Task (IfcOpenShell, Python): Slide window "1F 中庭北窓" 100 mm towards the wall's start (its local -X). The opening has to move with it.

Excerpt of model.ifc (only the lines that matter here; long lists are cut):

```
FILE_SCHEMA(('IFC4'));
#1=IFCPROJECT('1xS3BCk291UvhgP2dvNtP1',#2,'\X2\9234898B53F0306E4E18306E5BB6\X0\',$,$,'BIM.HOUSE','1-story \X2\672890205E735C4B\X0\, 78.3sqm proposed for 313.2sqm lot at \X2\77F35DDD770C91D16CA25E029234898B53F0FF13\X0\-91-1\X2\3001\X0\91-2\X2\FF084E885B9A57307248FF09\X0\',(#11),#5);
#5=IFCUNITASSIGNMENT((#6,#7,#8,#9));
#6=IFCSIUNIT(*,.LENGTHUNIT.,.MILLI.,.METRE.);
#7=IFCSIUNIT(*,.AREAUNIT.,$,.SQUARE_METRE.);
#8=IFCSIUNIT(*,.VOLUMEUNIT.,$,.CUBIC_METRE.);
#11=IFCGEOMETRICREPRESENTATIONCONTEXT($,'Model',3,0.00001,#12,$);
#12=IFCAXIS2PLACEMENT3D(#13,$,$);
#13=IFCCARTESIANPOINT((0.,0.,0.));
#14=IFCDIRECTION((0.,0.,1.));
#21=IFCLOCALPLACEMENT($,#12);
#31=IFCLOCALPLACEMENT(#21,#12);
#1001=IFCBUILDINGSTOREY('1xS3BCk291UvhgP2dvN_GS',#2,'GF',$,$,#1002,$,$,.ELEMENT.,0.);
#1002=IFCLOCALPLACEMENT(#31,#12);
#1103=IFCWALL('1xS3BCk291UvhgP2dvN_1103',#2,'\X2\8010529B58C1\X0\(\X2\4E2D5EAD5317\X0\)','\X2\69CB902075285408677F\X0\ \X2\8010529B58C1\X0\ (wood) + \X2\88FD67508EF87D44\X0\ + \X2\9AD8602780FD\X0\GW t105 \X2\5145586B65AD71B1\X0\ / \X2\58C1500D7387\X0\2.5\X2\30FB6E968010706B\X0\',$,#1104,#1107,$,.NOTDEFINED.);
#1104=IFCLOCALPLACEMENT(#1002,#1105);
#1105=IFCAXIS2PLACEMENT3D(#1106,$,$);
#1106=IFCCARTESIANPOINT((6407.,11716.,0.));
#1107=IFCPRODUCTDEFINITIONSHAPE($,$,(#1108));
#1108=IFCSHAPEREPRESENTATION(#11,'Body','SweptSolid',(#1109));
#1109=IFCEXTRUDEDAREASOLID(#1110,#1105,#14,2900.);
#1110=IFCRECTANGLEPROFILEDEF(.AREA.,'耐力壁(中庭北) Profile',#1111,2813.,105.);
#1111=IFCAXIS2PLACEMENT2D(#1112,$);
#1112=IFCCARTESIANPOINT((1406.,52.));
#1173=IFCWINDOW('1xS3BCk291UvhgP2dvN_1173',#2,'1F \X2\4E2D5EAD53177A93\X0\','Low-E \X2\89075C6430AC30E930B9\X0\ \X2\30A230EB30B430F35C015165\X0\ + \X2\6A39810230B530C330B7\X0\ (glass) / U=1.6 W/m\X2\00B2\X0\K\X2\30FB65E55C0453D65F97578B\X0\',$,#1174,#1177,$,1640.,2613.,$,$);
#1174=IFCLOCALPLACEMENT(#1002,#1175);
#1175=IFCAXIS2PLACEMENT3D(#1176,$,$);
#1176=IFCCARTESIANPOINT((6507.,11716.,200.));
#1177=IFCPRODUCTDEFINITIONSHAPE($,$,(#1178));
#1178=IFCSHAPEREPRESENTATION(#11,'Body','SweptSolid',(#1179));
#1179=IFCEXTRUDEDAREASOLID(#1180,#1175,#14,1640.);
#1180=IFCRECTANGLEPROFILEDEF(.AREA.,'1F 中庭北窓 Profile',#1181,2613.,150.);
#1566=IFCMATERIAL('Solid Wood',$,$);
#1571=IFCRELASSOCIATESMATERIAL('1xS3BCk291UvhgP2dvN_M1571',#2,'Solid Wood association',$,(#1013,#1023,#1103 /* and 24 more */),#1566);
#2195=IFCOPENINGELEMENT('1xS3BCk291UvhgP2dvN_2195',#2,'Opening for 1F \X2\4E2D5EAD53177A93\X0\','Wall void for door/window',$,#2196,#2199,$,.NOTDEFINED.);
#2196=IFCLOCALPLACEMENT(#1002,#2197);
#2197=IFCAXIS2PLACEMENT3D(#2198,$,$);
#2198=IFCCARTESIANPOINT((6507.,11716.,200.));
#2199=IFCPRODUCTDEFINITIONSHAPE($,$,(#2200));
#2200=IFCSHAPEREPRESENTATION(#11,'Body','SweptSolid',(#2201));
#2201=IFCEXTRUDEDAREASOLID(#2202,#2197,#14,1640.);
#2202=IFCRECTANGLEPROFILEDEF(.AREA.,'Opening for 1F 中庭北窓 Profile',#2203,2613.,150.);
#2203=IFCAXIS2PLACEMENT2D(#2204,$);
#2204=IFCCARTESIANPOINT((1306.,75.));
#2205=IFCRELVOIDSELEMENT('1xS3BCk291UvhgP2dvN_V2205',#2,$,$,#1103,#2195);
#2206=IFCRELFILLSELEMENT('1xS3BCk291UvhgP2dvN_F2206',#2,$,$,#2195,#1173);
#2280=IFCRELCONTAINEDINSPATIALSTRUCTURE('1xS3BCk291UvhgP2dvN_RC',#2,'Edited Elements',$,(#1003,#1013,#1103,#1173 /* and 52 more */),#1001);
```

```python
import ifcopenshell
import ifcopenshell.api.geometry
import ifcopenshell.util.placement
import ifcopenshell.util.unit

model = ifcopenshell.open("model.ifc")
unit_scale = ifcopenshell.util.unit.calculate_unit_scale(model)

window = model.by_guid("1xS3BCk291UvhgP2dvN_1173")
opening = window.FillsVoids[0].RelatingOpeningElement
wall = opening.VoidsElements[0].RelatingBuildingElement

wall_matrix = ifcopenshell.util.placement.get_local_placement(wall.ObjectPlacement)
shift = wall_matrix[:3, 0] * -0.1 / unit_scale
before = ifcopenshell.util.placement.get_local_placement(window.ObjectPlacement)[:3, 3].copy()

# The window is not placed relative to its opening, so move both.
for product in (opening, window):
    matrix = ifcopenshell.util.placement.get_local_placement(product.ObjectPlacement)
    matrix[:3, 3] += shift
    ifcopenshell.api.geometry.edit_object_placement(model, product=product, matrix=matrix, is_si=False)

after = ifcopenshell.util.placement.get_local_placement(window.ObjectPlacement)[:3, 3]
print("window moved by", (after - before).round(3) + 0.0)

model.write("model-out.ifc")
```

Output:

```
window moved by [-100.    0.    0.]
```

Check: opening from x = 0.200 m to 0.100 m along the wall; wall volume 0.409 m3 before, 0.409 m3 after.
